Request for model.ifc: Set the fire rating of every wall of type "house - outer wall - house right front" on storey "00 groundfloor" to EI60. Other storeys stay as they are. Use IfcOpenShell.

First a look at what the model holds.

```python
import ifcopenshell
import ifcopenshell.util.element

model = ifcopenshell.open("model.ifc")
print(model.schema)
storey = next(s for s in model.by_type("IfcBuildingStorey") if s.Name == "00 groundfloor")
walls = [e for e in ifcopenshell.util.element.get_decomposition(storey) if e.is_a("IfcWall")]
seen = {}
for e in walls:
    element_type = ifcopenshell.util.element.get_type(e)
    key = (element_type.Name if element_type != e and element_type else None, ifcopenshell.util.element.get_pset(e, "Pset_WallCommon", "FireRating"))
    seen[key] = seen.get(key, 0) + 1
for (name, value), count in sorted(seen.items(), key=str):
    print(count, "x", name, "|", value)
```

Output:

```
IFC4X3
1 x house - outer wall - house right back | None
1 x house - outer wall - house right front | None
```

```python
import ifcopenshell
import ifcopenshell.api.pset
import ifcopenshell.util.element

model = ifcopenshell.open("model.ifc")

storey = next(s for s in model.by_type("IfcBuildingStorey") if s.Name == "00 groundfloor")
walls = [e for e in ifcopenshell.util.element.get_decomposition(storey) if e.is_a("IfcWall")]

count = 0
for e in walls:
    element_type = ifcopenshell.util.element.get_type(e)
    if element_type in (None, e) or element_type.Name != "house - outer wall - house right front":
        continue
    # add_pset returns the element's existing set when there is one.
    pset = ifcopenshell.api.pset.add_pset(model, product=e, name="Pset_WallCommon")
    ifcopenshell.api.pset.edit_pset(model, pset=pset, properties={"FireRating": "EI60"})
    count += 1

print(count, "walls updated")

model.write("model_rev.ifc")
```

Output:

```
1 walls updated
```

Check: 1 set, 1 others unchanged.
